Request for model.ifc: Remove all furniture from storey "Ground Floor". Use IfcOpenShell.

First a look at what the model holds.

```python
import ifcopenshell
import ifcopenshell.util.element

model = ifcopenshell.open("model.ifc")
print(model.schema)
storey = next(s for s in model.by_type("IfcBuildingStorey") if s.Name == "Ground Floor")
furniture = [e for e in ifcopenshell.util.element.get_decomposition(storey) if e.is_a("IfcFurnishingElement")]
seen = {}
for e in furniture:
    element_type = ifcopenshell.util.element.get_type(e)
    name = element_type.Name if element_type not in (None, e) else None
    seen[name] = seen.get(name, 0) + 1
for name, count in sorted(seen.items(), key=str):
    print(count, "x", name)
```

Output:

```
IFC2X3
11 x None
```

```python
import ifcopenshell
import ifcopenshell.api.root
import ifcopenshell.util.element

model = ifcopenshell.open("model.ifc")

storey = next(s for s in model.by_type("IfcBuildingStorey") if s.Name == "Ground Floor")
furniture = [e for e in ifcopenshell.util.element.get_decomposition(storey) if e.is_a("IfcFurnishingElement")]

for e in furniture:
    ifcopenshell.api.root.remove_product(model, product=e)
print(len(furniture), "removed")

model.write("model_edited.ifc")
```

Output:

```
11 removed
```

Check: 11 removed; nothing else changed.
